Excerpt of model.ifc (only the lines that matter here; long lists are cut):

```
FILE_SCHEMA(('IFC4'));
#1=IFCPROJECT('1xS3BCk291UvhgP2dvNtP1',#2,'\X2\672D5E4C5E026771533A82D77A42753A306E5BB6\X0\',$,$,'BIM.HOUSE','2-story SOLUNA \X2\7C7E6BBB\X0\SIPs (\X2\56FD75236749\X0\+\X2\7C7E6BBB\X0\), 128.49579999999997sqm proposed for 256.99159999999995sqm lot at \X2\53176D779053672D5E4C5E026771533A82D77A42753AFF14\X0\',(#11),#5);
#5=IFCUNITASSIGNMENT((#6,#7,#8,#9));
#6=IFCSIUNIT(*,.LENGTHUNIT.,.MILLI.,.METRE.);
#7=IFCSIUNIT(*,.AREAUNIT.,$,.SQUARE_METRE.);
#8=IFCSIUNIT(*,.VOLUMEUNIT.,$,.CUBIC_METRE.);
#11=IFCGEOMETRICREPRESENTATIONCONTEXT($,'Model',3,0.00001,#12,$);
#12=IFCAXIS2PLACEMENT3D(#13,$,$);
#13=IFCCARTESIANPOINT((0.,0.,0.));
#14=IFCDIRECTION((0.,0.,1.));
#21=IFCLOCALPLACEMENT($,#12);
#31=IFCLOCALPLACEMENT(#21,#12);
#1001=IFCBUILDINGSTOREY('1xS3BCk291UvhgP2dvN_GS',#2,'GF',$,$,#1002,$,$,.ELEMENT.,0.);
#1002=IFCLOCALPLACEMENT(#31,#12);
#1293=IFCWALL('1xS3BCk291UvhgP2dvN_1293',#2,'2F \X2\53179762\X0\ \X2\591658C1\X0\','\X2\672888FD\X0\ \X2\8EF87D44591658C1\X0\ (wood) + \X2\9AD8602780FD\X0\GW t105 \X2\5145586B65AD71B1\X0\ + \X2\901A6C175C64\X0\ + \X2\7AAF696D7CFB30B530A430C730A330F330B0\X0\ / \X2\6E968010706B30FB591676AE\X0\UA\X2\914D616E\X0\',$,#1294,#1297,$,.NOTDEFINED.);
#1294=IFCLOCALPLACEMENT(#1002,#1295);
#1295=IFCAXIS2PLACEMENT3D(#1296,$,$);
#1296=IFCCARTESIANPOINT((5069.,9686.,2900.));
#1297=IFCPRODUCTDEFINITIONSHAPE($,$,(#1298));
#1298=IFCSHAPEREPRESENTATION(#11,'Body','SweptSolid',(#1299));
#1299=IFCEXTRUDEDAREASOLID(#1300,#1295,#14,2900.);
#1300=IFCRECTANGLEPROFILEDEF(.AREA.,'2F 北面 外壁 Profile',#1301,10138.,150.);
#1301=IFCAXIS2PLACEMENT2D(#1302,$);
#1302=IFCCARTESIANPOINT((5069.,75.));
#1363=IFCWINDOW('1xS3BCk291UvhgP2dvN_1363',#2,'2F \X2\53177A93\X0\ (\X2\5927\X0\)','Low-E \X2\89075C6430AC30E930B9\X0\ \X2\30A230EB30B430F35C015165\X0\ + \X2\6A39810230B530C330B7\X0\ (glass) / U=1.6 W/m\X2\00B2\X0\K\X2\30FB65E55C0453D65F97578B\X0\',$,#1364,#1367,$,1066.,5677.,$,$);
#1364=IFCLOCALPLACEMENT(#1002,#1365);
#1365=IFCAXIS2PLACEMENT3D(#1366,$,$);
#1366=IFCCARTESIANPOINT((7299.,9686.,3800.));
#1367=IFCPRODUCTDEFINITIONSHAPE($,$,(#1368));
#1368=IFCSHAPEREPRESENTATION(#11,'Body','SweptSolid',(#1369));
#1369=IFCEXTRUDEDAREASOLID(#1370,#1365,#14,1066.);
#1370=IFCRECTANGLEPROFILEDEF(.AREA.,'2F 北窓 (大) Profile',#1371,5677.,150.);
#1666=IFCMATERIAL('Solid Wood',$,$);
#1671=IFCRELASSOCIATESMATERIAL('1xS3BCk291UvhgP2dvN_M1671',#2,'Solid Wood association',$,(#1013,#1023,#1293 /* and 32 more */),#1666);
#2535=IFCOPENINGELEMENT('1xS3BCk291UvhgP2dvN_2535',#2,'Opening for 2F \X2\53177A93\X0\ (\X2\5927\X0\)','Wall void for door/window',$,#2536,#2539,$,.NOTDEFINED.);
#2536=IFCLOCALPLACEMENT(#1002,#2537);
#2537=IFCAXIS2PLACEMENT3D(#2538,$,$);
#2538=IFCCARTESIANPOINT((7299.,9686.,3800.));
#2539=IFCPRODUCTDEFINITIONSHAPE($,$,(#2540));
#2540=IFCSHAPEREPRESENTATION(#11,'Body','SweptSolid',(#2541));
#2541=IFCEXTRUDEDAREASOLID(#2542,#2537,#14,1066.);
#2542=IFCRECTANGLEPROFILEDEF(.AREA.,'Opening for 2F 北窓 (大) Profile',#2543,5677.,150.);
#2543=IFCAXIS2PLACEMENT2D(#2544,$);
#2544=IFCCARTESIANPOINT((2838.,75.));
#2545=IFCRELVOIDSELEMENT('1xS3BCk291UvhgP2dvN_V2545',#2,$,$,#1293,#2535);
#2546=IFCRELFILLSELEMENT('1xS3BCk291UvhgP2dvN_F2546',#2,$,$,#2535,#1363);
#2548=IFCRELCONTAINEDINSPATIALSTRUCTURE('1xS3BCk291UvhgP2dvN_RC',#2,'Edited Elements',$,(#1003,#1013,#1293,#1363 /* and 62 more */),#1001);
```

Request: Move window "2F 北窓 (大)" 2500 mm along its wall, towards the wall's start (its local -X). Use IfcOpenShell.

```python
import ifcopenshell
import ifcopenshell.api.geometry
import ifcopenshell.util.placement

model = ifcopenshell.open("model.ifc")

window = model.by_guid("1xS3BCk291UvhgP2dvN_1363")
opening = window.FillsVoids[0].RelatingOpeningElement
wall = opening.VoidsElements[0].RelatingBuildingElement

wall_matrix = ifcopenshell.util.placement.get_local_placement(wall.ObjectPlacement)
shift = wall_matrix[:3, 0] * -2500.0
before = ifcopenshell.util.placement.get_local_placement(window.ObjectPlacement)[:3, 3].copy()

# The window is not placed relative to its opening, so move both.
for product in (opening, window):
    matrix = ifcopenshell.util.placement.get_local_placement(product.ObjectPlacement)
    matrix[:3, 3] += shift
    ifcopenshell.api.geometry.edit_object_placement(model, product=product, matrix=matrix, is_si=False)

after = ifcopenshell.util.placement.get_local_placement(window.ObjectPlacement)[:3, 3]
print("window moved by", (after - before).round(3) + 0.0)

model.write("model_v2.ifc")
```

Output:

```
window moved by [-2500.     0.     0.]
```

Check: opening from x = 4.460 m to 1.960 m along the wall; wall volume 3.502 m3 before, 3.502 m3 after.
